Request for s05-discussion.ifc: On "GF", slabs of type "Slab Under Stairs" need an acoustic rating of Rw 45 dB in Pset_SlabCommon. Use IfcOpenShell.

First a look at what the model holds.

```python
import ifcopenshell
import ifcopenshell.util.element

model = ifcopenshell.open("s05-discussion.ifc")
print(model.schema)
storey = next(s for s in model.by_type("IfcBuildingStorey") if s.Name == "GF")
slabs = [e for e in ifcopenshell.util.element.get_decomposition(storey) if e.is_a("IfcSlab")]
seen = {}
for e in slabs:
    element_type = ifcopenshell.util.element.get_type(e)
    key = (element_type.Name if element_type != e and element_type else None, ifcopenshell.util.element.get_pset(e, "Pset_SlabCommon", "AcousticRating"))
    seen[key] = seen.get(key, 0) + 1
for (name, value), count in sorted(seen.items(), key=str):
    print(count, "x", name, "|", value)
```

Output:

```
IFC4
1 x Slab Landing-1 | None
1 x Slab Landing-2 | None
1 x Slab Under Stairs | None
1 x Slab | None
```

```python
import ifcopenshell
import ifcopenshell.api.pset
import ifcopenshell.util.element

model = ifcopenshell.open("s05-discussion.ifc")

storey = next(s for s in model.by_type("IfcBuildingStorey") if s.Name == "GF")
slabs = [e for e in ifcopenshell.util.element.get_decomposition(storey) if e.is_a("IfcSlab")]

count = 0
for e in slabs:
    element_type = ifcopenshell.util.element.get_type(e)
    if element_type in (None, e) or element_type.Name != "Slab Under Stairs":
        continue
    # add_pset returns the element's existing set when there is one.
    pset = ifcopenshell.api.pset.add_pset(model, product=e, name="Pset_SlabCommon")
    ifcopenshell.api.pset.edit_pset(model, pset=pset, properties={"AcousticRating": "Rw 45 dB"})
    count += 1

print(count, "slabs updated")

model.write("s05-discussion_rev.ifc")
```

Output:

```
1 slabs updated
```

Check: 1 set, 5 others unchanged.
